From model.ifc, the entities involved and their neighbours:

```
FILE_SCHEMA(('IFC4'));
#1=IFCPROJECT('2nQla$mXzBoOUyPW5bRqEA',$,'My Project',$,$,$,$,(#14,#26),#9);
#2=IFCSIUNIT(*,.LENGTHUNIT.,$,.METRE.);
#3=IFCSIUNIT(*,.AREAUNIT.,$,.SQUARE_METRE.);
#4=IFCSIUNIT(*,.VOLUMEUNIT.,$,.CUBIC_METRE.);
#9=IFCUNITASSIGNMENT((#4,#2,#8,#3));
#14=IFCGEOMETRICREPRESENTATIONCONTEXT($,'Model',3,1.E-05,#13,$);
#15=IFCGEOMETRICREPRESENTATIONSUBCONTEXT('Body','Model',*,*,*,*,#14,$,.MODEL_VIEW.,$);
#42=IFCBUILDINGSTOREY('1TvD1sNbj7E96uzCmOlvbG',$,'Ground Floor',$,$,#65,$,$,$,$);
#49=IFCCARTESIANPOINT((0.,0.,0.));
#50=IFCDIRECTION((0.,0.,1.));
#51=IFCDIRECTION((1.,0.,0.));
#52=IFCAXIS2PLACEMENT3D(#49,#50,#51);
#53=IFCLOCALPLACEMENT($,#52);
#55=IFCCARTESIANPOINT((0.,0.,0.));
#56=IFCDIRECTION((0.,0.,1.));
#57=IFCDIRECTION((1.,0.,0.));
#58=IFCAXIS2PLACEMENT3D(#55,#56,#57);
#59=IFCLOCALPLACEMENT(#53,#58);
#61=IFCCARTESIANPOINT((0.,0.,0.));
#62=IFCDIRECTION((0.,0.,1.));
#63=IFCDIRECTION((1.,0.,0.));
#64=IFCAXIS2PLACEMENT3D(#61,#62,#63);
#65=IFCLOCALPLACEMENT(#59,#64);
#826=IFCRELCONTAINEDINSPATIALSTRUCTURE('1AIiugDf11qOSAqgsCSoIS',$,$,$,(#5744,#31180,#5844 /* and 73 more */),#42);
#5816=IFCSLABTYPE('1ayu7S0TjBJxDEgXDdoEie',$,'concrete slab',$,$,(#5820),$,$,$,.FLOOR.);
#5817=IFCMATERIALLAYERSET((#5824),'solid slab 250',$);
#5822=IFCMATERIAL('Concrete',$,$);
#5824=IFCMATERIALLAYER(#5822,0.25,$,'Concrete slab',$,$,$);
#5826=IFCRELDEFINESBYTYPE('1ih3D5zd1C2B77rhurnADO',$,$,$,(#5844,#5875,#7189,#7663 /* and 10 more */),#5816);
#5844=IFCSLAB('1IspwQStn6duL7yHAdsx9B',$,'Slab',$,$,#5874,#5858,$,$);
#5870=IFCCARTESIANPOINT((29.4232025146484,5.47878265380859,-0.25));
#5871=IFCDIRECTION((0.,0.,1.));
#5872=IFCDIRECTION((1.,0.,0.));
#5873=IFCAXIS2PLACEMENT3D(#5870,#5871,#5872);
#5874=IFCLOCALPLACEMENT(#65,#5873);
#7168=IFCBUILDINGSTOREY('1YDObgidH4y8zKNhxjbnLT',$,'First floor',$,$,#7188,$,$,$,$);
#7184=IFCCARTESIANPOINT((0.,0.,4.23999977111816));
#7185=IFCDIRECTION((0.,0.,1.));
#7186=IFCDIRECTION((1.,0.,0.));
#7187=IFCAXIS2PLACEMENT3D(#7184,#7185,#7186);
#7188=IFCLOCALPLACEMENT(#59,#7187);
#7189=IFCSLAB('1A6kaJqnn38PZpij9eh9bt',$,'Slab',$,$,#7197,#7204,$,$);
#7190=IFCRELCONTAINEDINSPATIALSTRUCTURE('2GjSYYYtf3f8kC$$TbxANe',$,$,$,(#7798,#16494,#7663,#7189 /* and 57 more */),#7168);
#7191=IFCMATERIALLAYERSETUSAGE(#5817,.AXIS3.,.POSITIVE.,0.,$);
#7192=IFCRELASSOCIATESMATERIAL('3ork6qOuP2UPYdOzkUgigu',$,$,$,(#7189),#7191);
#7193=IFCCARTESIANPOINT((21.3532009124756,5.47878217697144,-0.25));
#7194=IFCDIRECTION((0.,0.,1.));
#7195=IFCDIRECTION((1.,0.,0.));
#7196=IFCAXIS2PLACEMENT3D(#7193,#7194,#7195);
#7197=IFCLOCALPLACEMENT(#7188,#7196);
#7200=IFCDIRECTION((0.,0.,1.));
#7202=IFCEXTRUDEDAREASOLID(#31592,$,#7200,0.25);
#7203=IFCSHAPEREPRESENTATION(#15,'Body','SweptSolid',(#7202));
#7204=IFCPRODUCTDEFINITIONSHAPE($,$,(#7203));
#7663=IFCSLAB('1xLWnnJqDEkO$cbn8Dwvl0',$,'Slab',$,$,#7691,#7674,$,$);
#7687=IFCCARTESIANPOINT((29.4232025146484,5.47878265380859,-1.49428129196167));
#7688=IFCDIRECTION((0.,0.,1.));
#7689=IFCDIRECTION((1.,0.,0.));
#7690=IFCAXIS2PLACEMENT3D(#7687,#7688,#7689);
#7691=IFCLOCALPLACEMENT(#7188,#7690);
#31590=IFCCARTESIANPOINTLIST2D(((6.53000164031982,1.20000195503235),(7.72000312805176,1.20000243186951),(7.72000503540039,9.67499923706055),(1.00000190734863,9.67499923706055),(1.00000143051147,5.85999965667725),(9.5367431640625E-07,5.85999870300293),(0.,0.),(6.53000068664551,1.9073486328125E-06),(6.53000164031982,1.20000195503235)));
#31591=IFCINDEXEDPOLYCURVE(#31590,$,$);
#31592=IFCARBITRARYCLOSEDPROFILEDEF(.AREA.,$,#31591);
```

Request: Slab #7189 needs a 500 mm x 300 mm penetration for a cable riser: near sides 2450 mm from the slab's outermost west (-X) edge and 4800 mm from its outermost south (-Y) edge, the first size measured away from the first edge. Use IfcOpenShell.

```python
import numpy as np
import ifcopenshell
import ifcopenshell.api.feature
import ifcopenshell.api.geometry
import ifcopenshell.api.root
import ifcopenshell.geom
import ifcopenshell.util.placement
import ifcopenshell.util.representation
import ifcopenshell.util.shape
import ifcopenshell.util.unit

model = ifcopenshell.open("model.ifc")
unit_scale = ifcopenshell.util.unit.calculate_unit_scale(model)
settings = ifcopenshell.geom.settings()


def volume(element):
    """Net volume in cubic metres, openings subtracted."""
    shape = ifcopenshell.geom.create_shape(settings, element)
    return ifcopenshell.util.shape.get_volume(shape.geometry)


slab = model.by_guid("1A6kaJqnn38PZpij9eh9bt")
before = volume(slab)

# Extent in the slab's own axes, in metres. The edges named are its -X and -Y sides.
slab_shape = ifcopenshell.geom.create_shape(settings, slab)
vertices = ifcopenshell.util.shape.get_vertices(slab_shape.geometry)
x_min, y_min, bottom = vertices.min(axis=0)
top = vertices[:, 2].max()

opening = ifcopenshell.api.root.create_entity(model, ifc_class="IfcOpeningElement", name="Cable riser opening", predefined_type="OPENING")
context = ifcopenshell.util.representation.get_context(model, "Model", "Body", "MODEL_VIEW")
width, depth = 0.5, 0.3
outline = [(0.0, 0.0), (width, 0.0), (width, depth), (0.0, depth), (0.0, 0.0)]
# Overshoot both faces by 50 mm so the cut is clean.
shape = ifcopenshell.api.geometry.add_slab_representation(
    model, context=context, depth=top - bottom + 0.1, polyline=outline
)
ifcopenshell.api.geometry.assign_representation(model, product=opening, representation=shape)

matrix = ifcopenshell.util.placement.get_local_placement(slab.ObjectPlacement)
matrix[:, 3] = matrix @ np.append(np.array([x_min + 2.45, y_min + 4.8, bottom - 0.05]) / unit_scale, 1.0)
ifcopenshell.api.geometry.edit_object_placement(model, product=opening, matrix=matrix, is_si=False)
ifcopenshell.api.feature.add_feature(model, feature=opening, element=slab)

after = volume(slab)

print(f"slab volume {before:.3f} -> {after:.3f} m3")

model.write("model_rev.ifc")
```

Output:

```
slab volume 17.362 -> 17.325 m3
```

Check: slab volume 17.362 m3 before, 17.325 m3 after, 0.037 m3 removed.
